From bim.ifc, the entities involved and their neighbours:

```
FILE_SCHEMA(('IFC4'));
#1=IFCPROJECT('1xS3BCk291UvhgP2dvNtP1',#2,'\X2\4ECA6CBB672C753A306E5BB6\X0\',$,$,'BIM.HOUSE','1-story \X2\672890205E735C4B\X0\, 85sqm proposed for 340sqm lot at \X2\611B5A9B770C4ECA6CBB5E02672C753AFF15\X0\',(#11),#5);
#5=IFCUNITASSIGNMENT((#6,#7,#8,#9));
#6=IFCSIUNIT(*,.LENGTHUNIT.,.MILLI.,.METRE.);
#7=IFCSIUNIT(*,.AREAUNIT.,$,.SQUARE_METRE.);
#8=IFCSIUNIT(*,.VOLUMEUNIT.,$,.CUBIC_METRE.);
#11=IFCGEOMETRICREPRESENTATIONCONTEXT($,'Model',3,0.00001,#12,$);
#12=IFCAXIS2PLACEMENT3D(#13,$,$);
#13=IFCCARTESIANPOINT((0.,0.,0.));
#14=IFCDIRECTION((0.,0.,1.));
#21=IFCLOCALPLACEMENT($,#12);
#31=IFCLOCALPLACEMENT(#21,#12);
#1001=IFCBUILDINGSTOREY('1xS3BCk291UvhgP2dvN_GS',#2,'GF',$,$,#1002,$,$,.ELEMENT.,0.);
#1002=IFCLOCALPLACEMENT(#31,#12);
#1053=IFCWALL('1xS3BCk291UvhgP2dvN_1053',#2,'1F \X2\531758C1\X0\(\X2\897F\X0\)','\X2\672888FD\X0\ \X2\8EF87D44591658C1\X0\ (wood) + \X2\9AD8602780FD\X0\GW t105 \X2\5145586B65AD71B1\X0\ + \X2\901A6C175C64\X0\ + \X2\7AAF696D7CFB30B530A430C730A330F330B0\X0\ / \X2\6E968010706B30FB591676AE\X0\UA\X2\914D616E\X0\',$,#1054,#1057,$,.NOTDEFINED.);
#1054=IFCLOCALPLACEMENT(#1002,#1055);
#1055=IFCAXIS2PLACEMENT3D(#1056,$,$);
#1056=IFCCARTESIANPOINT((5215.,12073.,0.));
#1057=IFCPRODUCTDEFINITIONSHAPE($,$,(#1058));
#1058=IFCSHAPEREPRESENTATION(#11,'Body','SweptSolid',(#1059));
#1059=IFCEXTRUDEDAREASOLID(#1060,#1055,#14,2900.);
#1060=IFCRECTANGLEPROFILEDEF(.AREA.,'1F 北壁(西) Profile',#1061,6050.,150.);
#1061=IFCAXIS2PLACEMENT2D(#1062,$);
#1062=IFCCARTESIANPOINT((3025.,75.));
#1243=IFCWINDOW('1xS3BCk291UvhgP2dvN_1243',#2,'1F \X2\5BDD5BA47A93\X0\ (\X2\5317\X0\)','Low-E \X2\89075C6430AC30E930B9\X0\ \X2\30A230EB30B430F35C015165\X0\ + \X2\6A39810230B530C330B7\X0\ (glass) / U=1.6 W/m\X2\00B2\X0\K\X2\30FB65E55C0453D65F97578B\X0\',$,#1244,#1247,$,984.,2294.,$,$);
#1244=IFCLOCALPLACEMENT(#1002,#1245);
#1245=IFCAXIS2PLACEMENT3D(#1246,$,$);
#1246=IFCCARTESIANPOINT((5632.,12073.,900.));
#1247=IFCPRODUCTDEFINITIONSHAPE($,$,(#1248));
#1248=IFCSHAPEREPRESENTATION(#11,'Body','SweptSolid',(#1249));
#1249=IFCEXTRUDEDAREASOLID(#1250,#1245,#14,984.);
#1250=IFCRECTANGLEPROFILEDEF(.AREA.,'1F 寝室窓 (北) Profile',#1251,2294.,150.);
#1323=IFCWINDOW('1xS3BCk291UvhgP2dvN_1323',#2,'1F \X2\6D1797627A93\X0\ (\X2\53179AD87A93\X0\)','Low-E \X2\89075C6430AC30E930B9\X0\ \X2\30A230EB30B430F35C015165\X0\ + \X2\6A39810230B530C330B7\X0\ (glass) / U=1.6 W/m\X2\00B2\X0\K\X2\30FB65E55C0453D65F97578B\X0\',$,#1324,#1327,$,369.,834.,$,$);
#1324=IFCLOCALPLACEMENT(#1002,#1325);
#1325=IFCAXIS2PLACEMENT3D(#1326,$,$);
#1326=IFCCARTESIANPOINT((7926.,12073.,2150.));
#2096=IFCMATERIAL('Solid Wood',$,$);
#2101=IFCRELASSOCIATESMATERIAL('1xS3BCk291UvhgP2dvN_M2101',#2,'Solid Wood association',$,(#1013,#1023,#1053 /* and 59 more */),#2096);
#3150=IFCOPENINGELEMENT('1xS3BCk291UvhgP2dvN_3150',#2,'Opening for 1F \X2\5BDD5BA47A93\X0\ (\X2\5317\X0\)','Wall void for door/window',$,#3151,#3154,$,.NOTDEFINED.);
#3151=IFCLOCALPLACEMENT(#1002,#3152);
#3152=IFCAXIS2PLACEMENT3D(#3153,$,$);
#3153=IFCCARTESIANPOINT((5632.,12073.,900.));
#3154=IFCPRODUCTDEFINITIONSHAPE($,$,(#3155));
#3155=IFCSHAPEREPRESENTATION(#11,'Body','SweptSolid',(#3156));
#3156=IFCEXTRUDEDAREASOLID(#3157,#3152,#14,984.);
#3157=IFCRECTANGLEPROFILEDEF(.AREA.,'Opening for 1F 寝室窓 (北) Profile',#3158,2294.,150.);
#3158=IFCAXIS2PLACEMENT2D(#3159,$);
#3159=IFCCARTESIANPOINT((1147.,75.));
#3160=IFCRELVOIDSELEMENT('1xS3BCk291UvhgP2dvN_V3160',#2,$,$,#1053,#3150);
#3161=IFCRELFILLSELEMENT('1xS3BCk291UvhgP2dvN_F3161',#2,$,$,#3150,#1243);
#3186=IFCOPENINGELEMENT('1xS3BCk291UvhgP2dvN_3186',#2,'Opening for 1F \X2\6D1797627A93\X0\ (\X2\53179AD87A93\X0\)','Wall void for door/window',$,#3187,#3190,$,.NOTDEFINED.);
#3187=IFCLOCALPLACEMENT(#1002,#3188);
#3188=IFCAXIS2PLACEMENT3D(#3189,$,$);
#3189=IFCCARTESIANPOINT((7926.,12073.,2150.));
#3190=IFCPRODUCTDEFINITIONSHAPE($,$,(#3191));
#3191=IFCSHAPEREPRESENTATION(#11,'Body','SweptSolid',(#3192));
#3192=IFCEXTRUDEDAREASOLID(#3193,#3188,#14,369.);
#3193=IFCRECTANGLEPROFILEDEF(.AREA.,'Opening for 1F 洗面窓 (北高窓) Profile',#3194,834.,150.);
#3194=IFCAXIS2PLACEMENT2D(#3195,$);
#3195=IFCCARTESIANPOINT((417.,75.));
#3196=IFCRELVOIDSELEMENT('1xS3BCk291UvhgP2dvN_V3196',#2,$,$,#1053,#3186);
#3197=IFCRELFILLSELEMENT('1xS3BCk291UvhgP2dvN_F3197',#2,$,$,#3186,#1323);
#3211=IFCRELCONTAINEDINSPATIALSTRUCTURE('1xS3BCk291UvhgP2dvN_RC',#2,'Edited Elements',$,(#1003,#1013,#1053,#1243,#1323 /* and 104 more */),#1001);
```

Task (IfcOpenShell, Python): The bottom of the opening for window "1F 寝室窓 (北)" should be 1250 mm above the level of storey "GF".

```python
import numpy as np
import ifcopenshell
import ifcopenshell.api.geometry
import ifcopenshell.geom
import ifcopenshell.util.element
import ifcopenshell.util.placement
import ifcopenshell.util.shape
import ifcopenshell.util.unit

model = ifcopenshell.open("bim.ifc")
unit_scale = ifcopenshell.util.unit.calculate_unit_scale(model)

window = model.by_id(1243)
opening = window.FillsVoids[0].RelatingOpeningElement
storey = ifcopenshell.util.element.get_container(window, ifc_class="IfcBuildingStorey")
level = ifcopenshell.util.placement.get_local_placement(storey.ObjectPlacement)[2, 3]

# The opening's origin need not be at the sill, so measure its lowest point.
shape = ifcopenshell.geom.create_shape(ifcopenshell.geom.settings(), opening)
bottom = ifcopenshell.util.shape.get_shape_bottom_elevation(shape, shape.geometry) / unit_scale
dz = level + 1.25 / unit_scale - bottom

shift = np.array([0.0, 0.0, dz])
# The window is not placed relative to its opening, so move both.
for product in (opening, window):
    matrix = ifcopenshell.util.placement.get_local_placement(product.ObjectPlacement)
    matrix[:3, 3] += shift
    ifcopenshell.api.geometry.edit_object_placement(model, product=product, matrix=matrix, is_si=False)

print(f"moved by {dz * unit_scale:+.3f} m")

model.write("bim_edited.ifc")
```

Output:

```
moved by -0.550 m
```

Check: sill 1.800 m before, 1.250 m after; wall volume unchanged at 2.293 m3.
